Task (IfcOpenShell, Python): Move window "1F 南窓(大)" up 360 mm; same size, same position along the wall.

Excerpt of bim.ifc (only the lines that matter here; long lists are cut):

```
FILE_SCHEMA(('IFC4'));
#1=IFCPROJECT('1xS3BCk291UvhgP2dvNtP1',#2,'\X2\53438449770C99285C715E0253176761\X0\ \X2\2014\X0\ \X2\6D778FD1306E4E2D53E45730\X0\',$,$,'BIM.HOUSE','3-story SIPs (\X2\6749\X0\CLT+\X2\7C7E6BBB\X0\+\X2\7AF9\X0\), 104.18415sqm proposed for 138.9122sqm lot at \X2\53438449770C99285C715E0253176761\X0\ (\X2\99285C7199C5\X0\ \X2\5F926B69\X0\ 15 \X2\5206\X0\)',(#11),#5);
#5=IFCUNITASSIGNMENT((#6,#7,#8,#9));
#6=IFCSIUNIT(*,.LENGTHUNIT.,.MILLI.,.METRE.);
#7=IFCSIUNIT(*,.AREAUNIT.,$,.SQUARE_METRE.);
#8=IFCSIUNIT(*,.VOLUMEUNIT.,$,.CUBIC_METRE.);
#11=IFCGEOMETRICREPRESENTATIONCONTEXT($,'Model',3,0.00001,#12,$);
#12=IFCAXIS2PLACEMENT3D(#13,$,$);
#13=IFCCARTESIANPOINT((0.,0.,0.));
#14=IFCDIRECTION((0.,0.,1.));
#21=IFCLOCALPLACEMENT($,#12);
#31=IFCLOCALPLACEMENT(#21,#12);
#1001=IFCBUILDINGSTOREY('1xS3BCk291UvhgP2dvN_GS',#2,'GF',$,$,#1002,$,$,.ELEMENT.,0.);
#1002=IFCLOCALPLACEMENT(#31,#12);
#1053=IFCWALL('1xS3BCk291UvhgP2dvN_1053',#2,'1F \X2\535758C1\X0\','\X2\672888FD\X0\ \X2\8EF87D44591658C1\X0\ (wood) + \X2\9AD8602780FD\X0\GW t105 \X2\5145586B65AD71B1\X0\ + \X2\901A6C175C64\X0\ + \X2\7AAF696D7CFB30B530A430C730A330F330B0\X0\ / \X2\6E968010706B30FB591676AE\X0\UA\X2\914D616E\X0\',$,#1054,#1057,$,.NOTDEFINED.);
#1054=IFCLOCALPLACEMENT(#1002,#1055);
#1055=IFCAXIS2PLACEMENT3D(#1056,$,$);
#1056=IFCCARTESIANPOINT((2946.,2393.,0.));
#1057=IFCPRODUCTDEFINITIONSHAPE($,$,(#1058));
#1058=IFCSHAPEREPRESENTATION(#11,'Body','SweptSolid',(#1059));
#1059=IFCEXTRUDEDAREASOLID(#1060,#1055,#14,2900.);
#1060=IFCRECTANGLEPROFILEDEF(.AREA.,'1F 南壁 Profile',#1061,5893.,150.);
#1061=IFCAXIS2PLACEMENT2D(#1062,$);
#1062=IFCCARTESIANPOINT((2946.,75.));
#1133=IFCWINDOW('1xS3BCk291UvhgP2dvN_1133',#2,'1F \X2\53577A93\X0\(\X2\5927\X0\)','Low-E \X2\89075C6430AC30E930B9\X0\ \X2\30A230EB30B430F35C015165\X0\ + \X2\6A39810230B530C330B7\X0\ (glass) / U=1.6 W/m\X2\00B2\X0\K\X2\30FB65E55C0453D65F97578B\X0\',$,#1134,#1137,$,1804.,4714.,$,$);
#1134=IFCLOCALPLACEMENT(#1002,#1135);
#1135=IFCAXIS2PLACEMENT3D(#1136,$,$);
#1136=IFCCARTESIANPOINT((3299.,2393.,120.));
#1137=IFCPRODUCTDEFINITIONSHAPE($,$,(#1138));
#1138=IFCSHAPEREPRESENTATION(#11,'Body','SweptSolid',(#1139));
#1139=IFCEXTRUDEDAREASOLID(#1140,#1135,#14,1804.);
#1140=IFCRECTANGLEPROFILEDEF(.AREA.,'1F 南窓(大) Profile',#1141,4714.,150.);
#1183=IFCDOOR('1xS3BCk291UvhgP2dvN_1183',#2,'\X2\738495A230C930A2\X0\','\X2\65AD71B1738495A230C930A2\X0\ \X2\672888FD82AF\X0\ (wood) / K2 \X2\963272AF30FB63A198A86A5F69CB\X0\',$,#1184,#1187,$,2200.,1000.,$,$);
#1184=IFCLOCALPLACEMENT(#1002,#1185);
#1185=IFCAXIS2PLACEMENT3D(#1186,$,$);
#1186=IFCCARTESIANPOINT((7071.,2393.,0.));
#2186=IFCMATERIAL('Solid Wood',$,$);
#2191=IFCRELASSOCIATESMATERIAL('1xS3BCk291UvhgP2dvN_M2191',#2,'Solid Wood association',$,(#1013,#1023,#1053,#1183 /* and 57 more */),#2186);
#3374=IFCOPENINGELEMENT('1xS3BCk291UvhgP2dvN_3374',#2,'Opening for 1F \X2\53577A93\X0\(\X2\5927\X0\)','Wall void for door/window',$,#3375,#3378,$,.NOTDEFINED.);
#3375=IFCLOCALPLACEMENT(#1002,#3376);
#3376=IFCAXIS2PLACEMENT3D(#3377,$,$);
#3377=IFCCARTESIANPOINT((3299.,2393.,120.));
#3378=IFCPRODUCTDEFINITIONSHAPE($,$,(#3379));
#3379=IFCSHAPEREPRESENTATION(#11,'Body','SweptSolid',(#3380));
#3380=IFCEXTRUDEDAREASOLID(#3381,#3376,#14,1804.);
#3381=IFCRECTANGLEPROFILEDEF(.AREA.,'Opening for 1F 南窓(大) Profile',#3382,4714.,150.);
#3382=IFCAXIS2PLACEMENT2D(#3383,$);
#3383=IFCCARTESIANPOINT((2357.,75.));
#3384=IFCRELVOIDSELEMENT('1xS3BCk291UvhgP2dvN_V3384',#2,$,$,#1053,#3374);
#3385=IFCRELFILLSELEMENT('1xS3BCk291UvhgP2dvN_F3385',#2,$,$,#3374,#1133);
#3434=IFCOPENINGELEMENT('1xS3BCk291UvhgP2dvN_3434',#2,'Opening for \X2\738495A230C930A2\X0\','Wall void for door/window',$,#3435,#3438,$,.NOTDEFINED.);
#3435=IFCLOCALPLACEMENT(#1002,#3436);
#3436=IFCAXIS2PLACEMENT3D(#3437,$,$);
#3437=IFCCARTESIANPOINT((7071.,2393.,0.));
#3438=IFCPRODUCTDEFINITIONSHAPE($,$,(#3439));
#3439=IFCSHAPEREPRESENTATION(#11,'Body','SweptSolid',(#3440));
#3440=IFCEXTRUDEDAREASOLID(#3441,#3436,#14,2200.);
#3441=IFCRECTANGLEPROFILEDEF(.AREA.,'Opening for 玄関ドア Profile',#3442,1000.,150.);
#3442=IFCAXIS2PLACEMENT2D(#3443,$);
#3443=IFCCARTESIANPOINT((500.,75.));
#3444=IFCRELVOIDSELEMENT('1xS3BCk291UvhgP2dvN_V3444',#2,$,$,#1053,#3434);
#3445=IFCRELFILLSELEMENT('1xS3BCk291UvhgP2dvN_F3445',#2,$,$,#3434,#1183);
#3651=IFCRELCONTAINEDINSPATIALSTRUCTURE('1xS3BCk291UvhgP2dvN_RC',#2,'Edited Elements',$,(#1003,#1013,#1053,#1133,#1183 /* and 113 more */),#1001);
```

```python
import numpy as np
import ifcopenshell
import ifcopenshell.api.geometry
import ifcopenshell.util.placement
import ifcopenshell.util.unit

model = ifcopenshell.open("bim.ifc")
unit_scale = ifcopenshell.util.unit.calculate_unit_scale(model)

window = model.by_id(1133)
opening = window.FillsVoids[0].RelatingOpeningElement
dz = 0.36 / unit_scale

shift = np.array([0.0, 0.0, dz])
# The window is not placed relative to its opening, so move both.
for product in (opening, window):
    matrix = ifcopenshell.util.placement.get_local_placement(product.ObjectPlacement)
    matrix[:3, 3] += shift
    ifcopenshell.api.geometry.edit_object_placement(model, product=product, matrix=matrix, is_si=False)

print(f"moved by {dz * unit_scale:+.3f} m")

model.write("bim_v2.ifc")
```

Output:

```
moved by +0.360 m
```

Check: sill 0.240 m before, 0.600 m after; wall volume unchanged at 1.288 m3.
